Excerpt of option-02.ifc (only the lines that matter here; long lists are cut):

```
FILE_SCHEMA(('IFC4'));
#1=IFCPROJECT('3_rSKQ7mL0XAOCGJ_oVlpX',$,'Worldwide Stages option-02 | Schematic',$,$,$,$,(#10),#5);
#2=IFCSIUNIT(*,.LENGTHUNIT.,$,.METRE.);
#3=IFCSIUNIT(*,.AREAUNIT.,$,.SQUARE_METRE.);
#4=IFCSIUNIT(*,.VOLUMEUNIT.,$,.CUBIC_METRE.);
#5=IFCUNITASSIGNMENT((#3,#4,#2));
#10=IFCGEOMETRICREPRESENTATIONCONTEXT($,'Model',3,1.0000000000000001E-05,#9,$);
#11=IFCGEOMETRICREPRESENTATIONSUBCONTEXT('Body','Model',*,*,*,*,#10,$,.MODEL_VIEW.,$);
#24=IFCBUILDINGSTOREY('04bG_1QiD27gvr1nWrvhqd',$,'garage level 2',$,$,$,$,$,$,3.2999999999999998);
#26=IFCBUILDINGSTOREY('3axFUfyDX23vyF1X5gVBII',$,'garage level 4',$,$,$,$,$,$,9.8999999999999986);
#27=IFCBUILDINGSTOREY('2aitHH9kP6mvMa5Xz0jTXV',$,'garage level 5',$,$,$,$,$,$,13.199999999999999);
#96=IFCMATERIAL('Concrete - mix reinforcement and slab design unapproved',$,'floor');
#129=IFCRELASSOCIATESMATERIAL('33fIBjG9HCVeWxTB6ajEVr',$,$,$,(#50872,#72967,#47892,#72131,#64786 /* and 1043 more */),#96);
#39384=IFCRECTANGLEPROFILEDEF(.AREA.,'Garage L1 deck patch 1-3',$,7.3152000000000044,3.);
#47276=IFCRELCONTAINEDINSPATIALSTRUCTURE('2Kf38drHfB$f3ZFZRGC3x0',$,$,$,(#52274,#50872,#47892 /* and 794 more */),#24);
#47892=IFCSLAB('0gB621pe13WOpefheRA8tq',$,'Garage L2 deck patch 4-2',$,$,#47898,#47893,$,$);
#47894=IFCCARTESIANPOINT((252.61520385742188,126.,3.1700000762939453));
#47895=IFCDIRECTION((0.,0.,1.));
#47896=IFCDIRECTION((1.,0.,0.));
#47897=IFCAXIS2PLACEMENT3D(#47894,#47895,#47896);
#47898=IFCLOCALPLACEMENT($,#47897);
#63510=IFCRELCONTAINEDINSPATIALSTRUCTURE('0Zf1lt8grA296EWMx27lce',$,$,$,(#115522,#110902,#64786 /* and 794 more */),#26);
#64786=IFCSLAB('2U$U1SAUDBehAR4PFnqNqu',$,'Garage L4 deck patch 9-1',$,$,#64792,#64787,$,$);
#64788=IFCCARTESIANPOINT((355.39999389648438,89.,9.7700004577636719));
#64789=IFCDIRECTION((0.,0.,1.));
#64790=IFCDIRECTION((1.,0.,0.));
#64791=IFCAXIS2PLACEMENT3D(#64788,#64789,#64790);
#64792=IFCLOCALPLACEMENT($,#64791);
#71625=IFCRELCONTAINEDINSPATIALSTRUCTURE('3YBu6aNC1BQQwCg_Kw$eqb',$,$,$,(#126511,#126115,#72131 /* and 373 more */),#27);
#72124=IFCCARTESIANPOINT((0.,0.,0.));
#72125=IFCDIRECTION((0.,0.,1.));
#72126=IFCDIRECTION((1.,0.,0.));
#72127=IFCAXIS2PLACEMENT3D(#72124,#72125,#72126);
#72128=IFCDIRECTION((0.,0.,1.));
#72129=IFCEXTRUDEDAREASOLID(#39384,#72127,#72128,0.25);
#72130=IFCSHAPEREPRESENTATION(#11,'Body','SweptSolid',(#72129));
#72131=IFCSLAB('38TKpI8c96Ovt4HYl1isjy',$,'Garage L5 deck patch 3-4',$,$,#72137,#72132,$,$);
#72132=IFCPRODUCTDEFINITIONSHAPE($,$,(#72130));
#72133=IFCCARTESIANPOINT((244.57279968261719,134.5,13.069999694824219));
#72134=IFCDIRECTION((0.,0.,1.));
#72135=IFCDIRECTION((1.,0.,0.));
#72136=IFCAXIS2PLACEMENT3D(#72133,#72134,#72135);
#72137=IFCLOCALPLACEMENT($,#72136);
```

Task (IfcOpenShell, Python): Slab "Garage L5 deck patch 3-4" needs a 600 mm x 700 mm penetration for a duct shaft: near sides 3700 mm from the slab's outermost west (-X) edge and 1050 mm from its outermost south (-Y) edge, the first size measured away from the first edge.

```python
import numpy as np
import ifcopenshell
import ifcopenshell.api.feature
import ifcopenshell.api.geometry
import ifcopenshell.api.root
import ifcopenshell.geom
import ifcopenshell.util.placement
import ifcopenshell.util.representation
import ifcopenshell.util.shape
import ifcopenshell.util.unit

model = ifcopenshell.open("option-02.ifc")
unit_scale = ifcopenshell.util.unit.calculate_unit_scale(model)
settings = ifcopenshell.geom.settings()


def volume(element):
    """Net volume in cubic metres, openings subtracted."""
    shape = ifcopenshell.geom.create_shape(settings, element)
    return ifcopenshell.util.shape.get_volume(shape.geometry)


slab = model.by_guid("38TKpI8c96Ovt4HYl1isjy")
before = volume(slab)

# Extent in the slab's own axes, in metres. The edges named are its -X and -Y sides.
slab_shape = ifcopenshell.geom.create_shape(settings, slab)
vertices = ifcopenshell.util.shape.get_vertices(slab_shape.geometry)
x_min, y_min, bottom = vertices.min(axis=0)
top = vertices[:, 2].max()

opening = ifcopenshell.api.root.create_entity(model, ifc_class="IfcOpeningElement", name="Duct shaft opening", predefined_type="OPENING")
context = ifcopenshell.util.representation.get_context(model, "Model", "Body", "MODEL_VIEW")
width, depth = 0.6, 0.7
outline = [(0.0, 0.0), (width, 0.0), (width, depth), (0.0, depth), (0.0, 0.0)]
# Overshoot both faces by 50 mm so the cut is clean.
shape = ifcopenshell.api.geometry.add_slab_representation(
    model, context=context, depth=top - bottom + 0.1, polyline=outline
)
ifcopenshell.api.geometry.assign_representation(model, product=opening, representation=shape)

matrix = ifcopenshell.util.placement.get_local_placement(slab.ObjectPlacement)
matrix[:, 3] = matrix @ np.append(np.array([x_min + 3.7, y_min + 1.05, bottom - 0.05]) / unit_scale, 1.0)
ifcopenshell.api.geometry.edit_object_placement(model, product=opening, matrix=matrix, is_si=False)
ifcopenshell.api.feature.add_feature(model, feature=opening, element=slab)

after = volume(slab)

print(f"slab volume {before:.3f} -> {after:.3f} m3")

model.write("option-02_rev.ifc")
```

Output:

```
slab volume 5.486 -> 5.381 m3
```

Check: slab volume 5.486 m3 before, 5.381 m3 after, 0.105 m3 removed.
